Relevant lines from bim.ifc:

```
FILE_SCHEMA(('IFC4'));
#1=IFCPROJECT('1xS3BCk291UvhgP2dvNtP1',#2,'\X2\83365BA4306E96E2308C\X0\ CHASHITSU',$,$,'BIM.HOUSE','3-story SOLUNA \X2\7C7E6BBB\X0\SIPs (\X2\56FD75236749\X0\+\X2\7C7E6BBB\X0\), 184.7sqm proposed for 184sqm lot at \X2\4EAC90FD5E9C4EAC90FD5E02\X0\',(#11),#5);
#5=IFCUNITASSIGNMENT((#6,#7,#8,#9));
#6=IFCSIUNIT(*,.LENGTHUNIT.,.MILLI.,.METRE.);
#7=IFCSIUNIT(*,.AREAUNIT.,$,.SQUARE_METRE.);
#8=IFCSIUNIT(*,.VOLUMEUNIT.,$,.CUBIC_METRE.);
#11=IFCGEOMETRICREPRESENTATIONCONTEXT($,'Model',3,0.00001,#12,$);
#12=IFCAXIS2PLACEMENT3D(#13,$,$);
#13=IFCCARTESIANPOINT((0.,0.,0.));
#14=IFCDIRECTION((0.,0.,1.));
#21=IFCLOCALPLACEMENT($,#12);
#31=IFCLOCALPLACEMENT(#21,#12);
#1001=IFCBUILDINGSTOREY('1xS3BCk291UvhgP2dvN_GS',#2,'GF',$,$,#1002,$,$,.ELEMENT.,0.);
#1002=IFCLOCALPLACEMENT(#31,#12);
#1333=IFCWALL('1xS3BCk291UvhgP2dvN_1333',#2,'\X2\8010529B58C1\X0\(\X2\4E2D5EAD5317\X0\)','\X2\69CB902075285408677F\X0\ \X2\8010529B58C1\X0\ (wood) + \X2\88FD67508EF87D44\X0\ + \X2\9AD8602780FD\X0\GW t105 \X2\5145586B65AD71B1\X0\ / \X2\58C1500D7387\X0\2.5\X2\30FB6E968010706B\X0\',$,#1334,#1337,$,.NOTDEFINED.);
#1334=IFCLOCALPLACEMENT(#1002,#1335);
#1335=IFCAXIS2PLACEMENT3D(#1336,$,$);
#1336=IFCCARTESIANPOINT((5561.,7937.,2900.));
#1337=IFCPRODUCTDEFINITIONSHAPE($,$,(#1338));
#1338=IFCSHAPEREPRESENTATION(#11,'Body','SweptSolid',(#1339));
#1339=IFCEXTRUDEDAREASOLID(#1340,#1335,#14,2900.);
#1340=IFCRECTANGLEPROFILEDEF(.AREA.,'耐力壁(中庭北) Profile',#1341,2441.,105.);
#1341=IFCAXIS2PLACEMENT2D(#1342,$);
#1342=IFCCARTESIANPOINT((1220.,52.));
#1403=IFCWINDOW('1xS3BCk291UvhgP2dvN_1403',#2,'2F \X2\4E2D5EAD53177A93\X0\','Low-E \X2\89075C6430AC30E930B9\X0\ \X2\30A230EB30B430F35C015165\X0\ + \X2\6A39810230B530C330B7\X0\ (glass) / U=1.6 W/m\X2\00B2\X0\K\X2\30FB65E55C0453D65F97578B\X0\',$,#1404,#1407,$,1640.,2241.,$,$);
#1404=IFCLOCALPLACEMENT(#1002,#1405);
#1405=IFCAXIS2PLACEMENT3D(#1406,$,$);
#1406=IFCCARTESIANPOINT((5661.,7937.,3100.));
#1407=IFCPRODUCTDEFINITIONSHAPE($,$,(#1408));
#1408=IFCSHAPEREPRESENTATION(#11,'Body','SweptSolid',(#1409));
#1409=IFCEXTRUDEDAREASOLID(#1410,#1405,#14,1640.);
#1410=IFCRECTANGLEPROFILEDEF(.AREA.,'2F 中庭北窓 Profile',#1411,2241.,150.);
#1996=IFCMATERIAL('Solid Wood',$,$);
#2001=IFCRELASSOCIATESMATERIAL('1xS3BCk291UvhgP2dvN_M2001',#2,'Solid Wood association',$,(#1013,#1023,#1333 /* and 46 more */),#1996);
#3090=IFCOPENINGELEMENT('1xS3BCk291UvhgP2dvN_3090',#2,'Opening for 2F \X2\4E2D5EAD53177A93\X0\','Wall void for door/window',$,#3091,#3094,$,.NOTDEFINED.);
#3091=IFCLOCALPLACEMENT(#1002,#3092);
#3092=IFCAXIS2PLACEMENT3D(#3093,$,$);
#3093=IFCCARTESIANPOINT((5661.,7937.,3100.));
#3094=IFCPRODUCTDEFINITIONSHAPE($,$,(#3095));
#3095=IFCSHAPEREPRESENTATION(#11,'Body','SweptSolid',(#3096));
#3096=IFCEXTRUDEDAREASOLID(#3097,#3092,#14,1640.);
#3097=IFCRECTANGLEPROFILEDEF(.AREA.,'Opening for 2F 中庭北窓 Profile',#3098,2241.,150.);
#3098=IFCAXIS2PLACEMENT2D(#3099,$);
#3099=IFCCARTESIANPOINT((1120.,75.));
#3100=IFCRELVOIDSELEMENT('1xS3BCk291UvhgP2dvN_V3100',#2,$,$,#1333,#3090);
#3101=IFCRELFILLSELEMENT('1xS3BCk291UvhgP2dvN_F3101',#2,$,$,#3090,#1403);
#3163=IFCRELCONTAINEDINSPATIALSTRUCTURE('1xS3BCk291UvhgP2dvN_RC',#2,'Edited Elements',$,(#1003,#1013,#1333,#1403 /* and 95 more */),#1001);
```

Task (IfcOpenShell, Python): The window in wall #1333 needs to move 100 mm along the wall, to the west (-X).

```python
import ifcopenshell
import ifcopenshell.api.geometry
import ifcopenshell.util.placement
import ifcopenshell.util.unit

model = ifcopenshell.open("bim.ifc")
unit_scale = ifcopenshell.util.unit.calculate_unit_scale(model)

window = model.by_guid("1xS3BCk291UvhgP2dvN_1403")
opening = window.FillsVoids[0].RelatingOpeningElement
wall = opening.VoidsElements[0].RelatingBuildingElement

wall_matrix = ifcopenshell.util.placement.get_local_placement(wall.ObjectPlacement)
shift = wall_matrix[:3, 0] * -0.1 / unit_scale
before = ifcopenshell.util.placement.get_local_placement(window.ObjectPlacement)[:3, 3].copy()

# The window is not placed relative to its opening, so move both.
for product in (opening, window):
    matrix = ifcopenshell.util.placement.get_local_placement(product.ObjectPlacement)
    matrix[:3, 3] += shift
    ifcopenshell.api.geometry.edit_object_placement(model, product=product, matrix=matrix, is_si=False)

after = ifcopenshell.util.placement.get_local_placement(window.ObjectPlacement)[:3, 3]
print("window moved by", (after - before).round(3) + 0.0)

model.write("bim_updated.ifc")
```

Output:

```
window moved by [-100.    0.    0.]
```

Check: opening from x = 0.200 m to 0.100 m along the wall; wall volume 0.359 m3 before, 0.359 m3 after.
